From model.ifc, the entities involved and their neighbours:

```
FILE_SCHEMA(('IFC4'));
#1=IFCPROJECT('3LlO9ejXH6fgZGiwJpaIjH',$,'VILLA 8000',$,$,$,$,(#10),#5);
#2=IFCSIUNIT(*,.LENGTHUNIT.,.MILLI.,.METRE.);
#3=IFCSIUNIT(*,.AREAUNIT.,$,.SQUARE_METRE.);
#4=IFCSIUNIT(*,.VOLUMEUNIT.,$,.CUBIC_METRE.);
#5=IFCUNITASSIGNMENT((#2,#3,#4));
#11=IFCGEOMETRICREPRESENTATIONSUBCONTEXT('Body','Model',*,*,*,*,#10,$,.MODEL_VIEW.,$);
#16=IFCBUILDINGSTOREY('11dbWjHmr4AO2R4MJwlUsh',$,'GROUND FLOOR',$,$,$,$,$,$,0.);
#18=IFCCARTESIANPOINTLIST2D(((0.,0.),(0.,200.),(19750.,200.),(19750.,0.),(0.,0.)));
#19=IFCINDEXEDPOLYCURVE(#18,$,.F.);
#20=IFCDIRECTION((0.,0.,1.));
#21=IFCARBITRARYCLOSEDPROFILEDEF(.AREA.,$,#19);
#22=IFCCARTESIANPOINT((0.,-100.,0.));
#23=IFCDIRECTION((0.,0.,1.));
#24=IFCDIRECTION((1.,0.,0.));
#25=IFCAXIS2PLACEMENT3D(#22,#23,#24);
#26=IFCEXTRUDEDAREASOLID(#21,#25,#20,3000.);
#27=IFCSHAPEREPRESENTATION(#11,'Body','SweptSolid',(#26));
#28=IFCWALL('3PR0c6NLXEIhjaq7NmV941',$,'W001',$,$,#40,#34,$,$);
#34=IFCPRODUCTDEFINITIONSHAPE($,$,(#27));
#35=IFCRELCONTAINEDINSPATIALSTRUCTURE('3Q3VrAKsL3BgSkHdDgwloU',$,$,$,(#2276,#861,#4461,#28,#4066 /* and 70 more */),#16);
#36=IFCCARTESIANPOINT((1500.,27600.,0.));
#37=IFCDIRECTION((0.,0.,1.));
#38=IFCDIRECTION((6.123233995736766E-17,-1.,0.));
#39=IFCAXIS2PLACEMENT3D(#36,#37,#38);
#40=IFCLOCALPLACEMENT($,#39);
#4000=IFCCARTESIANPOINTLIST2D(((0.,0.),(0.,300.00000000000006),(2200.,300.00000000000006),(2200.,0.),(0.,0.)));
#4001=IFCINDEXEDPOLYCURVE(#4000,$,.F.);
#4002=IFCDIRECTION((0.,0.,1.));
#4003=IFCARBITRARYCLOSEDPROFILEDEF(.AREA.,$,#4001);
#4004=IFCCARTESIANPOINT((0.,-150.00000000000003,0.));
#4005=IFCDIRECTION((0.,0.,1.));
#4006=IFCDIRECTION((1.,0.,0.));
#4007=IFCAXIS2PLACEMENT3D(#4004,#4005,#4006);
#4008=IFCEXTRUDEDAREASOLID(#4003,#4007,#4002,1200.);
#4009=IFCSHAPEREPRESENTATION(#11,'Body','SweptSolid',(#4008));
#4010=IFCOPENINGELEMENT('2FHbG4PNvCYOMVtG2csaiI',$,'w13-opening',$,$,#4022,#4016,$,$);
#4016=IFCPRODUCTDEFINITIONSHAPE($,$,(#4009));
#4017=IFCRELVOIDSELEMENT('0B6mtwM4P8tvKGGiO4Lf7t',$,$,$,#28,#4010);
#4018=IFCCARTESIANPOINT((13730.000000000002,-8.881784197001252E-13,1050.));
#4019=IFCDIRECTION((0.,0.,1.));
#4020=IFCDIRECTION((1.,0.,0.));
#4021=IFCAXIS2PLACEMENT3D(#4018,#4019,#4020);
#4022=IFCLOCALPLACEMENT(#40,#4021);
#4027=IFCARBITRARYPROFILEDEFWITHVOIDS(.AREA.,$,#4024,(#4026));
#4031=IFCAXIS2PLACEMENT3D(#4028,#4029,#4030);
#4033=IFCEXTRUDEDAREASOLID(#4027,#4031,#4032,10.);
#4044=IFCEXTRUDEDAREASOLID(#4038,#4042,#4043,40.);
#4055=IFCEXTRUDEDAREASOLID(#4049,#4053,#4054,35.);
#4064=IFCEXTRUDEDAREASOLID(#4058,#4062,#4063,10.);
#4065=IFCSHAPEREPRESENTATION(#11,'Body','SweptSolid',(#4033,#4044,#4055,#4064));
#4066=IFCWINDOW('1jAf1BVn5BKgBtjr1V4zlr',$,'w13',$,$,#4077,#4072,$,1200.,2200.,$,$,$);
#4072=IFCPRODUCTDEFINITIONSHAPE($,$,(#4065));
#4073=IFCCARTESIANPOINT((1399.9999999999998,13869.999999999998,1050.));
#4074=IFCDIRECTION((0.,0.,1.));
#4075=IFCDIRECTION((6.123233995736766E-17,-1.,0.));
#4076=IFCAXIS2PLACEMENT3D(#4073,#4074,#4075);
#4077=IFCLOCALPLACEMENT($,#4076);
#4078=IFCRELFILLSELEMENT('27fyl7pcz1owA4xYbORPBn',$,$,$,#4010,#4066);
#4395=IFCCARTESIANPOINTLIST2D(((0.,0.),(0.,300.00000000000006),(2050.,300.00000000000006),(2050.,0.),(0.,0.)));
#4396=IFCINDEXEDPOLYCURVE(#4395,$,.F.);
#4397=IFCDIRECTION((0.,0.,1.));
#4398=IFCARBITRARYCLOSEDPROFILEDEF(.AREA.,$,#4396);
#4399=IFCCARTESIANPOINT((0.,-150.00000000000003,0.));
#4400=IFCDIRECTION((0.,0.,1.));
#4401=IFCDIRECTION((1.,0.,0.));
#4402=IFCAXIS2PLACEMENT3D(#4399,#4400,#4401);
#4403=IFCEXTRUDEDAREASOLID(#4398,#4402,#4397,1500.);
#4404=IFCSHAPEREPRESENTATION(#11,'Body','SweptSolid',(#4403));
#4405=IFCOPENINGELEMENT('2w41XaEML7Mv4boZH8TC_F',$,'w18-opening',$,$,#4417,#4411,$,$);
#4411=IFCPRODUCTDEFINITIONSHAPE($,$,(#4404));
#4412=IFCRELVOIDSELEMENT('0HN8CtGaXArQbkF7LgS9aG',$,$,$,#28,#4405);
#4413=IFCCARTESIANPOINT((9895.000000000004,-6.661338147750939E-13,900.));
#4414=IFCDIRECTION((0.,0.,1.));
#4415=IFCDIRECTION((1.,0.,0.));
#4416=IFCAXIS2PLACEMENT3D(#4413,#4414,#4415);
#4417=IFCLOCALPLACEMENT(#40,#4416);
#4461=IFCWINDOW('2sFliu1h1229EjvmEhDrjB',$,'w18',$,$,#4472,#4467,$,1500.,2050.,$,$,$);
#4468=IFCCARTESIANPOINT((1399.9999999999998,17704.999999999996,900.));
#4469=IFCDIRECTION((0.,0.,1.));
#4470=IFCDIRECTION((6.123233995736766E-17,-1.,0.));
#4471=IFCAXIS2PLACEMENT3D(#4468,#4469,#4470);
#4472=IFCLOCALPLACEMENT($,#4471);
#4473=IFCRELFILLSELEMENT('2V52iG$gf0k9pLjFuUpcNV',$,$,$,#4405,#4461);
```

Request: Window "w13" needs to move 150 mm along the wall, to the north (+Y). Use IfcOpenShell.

```python
import ifcopenshell
import ifcopenshell.api.geometry
import ifcopenshell.util.placement

model = ifcopenshell.open("model.ifc")

window = model.by_id(4066)
opening = window.FillsVoids[0].RelatingOpeningElement
wall = opening.VoidsElements[0].RelatingBuildingElement

wall_matrix = ifcopenshell.util.placement.get_local_placement(wall.ObjectPlacement)
shift = wall_matrix[:3, 0] * -150.0
before = ifcopenshell.util.placement.get_local_placement(window.ObjectPlacement)[:3, 3].copy()

# The window is not placed relative to its opening, so move both.
for product in (opening, window):
    matrix = ifcopenshell.util.placement.get_local_placement(product.ObjectPlacement)
    matrix[:3, 3] += shift
    ifcopenshell.api.geometry.edit_object_placement(model, product=product, matrix=matrix, is_si=False)

after = ifcopenshell.util.placement.get_local_placement(window.ObjectPlacement)[:3, 3]
print("window moved by", (after - before).round(3) + 0.0)

model.write("model-out.ifc")
```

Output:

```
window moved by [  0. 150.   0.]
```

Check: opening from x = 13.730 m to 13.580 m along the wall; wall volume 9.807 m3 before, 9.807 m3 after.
